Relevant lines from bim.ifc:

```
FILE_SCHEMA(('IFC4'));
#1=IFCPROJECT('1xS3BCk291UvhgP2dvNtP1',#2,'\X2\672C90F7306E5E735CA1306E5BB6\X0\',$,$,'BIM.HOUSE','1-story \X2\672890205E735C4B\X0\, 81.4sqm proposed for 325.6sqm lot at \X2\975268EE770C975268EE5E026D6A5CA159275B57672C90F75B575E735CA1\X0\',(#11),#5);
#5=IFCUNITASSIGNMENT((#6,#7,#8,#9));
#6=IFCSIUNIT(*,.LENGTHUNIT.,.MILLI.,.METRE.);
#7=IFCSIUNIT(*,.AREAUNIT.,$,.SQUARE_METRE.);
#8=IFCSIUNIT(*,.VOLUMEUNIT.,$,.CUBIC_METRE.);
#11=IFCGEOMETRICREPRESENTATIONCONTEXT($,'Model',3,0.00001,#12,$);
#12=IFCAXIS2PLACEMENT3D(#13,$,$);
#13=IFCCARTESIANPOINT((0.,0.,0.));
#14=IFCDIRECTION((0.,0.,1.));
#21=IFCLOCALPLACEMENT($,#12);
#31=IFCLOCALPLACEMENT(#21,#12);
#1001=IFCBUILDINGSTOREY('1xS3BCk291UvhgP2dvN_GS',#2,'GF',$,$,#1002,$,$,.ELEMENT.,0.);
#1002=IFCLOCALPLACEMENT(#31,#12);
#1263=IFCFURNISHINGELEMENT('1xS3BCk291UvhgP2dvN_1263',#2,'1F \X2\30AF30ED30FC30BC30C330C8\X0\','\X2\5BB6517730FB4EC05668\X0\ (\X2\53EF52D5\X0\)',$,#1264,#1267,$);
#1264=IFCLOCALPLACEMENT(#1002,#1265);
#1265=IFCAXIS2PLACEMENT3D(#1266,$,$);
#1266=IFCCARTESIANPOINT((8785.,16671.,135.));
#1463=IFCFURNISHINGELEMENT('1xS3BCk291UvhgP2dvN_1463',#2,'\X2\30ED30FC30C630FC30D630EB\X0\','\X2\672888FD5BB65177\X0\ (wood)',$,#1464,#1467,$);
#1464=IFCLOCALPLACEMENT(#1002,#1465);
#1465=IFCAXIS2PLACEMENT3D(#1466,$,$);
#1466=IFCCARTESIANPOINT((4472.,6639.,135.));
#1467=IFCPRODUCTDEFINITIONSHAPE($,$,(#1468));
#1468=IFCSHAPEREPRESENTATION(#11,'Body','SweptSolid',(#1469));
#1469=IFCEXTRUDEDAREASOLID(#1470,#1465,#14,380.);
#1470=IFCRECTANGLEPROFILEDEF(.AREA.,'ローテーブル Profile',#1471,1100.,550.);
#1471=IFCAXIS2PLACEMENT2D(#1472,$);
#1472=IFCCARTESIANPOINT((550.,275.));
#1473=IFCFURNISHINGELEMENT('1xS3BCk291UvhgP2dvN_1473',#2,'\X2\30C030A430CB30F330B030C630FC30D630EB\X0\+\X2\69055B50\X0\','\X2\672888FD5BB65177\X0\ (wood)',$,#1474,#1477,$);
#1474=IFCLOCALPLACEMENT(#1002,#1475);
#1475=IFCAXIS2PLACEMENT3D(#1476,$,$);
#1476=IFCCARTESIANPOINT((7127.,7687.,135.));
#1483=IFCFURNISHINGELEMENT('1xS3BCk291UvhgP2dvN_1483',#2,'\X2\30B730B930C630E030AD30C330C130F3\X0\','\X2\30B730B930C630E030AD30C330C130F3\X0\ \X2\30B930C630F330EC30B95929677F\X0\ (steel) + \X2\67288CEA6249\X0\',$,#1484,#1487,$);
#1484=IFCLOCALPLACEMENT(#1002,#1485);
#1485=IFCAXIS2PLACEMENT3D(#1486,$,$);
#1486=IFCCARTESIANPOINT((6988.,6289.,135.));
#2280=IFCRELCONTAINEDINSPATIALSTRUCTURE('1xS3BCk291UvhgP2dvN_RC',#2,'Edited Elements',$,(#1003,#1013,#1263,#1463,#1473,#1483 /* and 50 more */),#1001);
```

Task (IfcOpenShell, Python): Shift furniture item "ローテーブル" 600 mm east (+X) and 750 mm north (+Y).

```python
import ifcopenshell
import ifcopenshell.api.geometry
import ifcopenshell.util.placement
import ifcopenshell.util.unit

model = ifcopenshell.open("bim.ifc")
unit_scale = ifcopenshell.util.unit.calculate_unit_scale(model)

item = model.by_id(1463)
matrix = ifcopenshell.util.placement.get_local_placement(item.ObjectPlacement)
matrix[0, 3] += 0.6 / unit_scale
matrix[1, 3] += 0.75 / unit_scale
ifcopenshell.api.geometry.edit_object_placement(model, product=item, matrix=matrix, is_si=False)

print(ifcopenshell.util.placement.get_local_placement(item.ObjectPlacement).round(3) + 0.0)

model.write("bim_v2.ifc")
```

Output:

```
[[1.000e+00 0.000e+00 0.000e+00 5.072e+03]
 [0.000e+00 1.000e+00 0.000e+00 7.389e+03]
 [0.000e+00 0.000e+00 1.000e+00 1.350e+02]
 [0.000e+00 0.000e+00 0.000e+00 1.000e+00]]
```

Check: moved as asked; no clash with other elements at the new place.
